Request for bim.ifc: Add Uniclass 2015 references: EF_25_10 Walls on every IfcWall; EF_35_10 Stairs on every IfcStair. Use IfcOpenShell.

First a look at what the model holds.

```python
import ifcopenshell

model = ifcopenshell.open("bim.ifc")
print(model.schema)
print("classifications:", [c.Name for c in model.by_type("IfcClassification")])
for ifc_class in ("IfcDoor", "IfcRoof", "IfcStair", "IfcWall", "IfcWindow"):
    print(ifc_class, len(model.by_type(ifc_class)))
```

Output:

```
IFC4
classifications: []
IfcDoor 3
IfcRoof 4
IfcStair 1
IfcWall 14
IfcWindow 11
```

```python
import ifcopenshell
import ifcopenshell.api.classification

model = ifcopenshell.open("bim.ifc")

system = ifcopenshell.api.classification.add_classification(model, classification="Uniclass 2015")

codes = {
    "IfcWall": ("EF_25_10", "Walls"),
    "IfcStair": ("EF_35_10", "Stairs"),
}
for ifc_class, (code, name) in codes.items():
    products = model.by_type(ifc_class)
    ifcopenshell.api.classification.add_reference(
        model, products=products, classification=system, identification=code, name=name
    )
    print(code, len(products))

model.write("bim_v2.ifc")
```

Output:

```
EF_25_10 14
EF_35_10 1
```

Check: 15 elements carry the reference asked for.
